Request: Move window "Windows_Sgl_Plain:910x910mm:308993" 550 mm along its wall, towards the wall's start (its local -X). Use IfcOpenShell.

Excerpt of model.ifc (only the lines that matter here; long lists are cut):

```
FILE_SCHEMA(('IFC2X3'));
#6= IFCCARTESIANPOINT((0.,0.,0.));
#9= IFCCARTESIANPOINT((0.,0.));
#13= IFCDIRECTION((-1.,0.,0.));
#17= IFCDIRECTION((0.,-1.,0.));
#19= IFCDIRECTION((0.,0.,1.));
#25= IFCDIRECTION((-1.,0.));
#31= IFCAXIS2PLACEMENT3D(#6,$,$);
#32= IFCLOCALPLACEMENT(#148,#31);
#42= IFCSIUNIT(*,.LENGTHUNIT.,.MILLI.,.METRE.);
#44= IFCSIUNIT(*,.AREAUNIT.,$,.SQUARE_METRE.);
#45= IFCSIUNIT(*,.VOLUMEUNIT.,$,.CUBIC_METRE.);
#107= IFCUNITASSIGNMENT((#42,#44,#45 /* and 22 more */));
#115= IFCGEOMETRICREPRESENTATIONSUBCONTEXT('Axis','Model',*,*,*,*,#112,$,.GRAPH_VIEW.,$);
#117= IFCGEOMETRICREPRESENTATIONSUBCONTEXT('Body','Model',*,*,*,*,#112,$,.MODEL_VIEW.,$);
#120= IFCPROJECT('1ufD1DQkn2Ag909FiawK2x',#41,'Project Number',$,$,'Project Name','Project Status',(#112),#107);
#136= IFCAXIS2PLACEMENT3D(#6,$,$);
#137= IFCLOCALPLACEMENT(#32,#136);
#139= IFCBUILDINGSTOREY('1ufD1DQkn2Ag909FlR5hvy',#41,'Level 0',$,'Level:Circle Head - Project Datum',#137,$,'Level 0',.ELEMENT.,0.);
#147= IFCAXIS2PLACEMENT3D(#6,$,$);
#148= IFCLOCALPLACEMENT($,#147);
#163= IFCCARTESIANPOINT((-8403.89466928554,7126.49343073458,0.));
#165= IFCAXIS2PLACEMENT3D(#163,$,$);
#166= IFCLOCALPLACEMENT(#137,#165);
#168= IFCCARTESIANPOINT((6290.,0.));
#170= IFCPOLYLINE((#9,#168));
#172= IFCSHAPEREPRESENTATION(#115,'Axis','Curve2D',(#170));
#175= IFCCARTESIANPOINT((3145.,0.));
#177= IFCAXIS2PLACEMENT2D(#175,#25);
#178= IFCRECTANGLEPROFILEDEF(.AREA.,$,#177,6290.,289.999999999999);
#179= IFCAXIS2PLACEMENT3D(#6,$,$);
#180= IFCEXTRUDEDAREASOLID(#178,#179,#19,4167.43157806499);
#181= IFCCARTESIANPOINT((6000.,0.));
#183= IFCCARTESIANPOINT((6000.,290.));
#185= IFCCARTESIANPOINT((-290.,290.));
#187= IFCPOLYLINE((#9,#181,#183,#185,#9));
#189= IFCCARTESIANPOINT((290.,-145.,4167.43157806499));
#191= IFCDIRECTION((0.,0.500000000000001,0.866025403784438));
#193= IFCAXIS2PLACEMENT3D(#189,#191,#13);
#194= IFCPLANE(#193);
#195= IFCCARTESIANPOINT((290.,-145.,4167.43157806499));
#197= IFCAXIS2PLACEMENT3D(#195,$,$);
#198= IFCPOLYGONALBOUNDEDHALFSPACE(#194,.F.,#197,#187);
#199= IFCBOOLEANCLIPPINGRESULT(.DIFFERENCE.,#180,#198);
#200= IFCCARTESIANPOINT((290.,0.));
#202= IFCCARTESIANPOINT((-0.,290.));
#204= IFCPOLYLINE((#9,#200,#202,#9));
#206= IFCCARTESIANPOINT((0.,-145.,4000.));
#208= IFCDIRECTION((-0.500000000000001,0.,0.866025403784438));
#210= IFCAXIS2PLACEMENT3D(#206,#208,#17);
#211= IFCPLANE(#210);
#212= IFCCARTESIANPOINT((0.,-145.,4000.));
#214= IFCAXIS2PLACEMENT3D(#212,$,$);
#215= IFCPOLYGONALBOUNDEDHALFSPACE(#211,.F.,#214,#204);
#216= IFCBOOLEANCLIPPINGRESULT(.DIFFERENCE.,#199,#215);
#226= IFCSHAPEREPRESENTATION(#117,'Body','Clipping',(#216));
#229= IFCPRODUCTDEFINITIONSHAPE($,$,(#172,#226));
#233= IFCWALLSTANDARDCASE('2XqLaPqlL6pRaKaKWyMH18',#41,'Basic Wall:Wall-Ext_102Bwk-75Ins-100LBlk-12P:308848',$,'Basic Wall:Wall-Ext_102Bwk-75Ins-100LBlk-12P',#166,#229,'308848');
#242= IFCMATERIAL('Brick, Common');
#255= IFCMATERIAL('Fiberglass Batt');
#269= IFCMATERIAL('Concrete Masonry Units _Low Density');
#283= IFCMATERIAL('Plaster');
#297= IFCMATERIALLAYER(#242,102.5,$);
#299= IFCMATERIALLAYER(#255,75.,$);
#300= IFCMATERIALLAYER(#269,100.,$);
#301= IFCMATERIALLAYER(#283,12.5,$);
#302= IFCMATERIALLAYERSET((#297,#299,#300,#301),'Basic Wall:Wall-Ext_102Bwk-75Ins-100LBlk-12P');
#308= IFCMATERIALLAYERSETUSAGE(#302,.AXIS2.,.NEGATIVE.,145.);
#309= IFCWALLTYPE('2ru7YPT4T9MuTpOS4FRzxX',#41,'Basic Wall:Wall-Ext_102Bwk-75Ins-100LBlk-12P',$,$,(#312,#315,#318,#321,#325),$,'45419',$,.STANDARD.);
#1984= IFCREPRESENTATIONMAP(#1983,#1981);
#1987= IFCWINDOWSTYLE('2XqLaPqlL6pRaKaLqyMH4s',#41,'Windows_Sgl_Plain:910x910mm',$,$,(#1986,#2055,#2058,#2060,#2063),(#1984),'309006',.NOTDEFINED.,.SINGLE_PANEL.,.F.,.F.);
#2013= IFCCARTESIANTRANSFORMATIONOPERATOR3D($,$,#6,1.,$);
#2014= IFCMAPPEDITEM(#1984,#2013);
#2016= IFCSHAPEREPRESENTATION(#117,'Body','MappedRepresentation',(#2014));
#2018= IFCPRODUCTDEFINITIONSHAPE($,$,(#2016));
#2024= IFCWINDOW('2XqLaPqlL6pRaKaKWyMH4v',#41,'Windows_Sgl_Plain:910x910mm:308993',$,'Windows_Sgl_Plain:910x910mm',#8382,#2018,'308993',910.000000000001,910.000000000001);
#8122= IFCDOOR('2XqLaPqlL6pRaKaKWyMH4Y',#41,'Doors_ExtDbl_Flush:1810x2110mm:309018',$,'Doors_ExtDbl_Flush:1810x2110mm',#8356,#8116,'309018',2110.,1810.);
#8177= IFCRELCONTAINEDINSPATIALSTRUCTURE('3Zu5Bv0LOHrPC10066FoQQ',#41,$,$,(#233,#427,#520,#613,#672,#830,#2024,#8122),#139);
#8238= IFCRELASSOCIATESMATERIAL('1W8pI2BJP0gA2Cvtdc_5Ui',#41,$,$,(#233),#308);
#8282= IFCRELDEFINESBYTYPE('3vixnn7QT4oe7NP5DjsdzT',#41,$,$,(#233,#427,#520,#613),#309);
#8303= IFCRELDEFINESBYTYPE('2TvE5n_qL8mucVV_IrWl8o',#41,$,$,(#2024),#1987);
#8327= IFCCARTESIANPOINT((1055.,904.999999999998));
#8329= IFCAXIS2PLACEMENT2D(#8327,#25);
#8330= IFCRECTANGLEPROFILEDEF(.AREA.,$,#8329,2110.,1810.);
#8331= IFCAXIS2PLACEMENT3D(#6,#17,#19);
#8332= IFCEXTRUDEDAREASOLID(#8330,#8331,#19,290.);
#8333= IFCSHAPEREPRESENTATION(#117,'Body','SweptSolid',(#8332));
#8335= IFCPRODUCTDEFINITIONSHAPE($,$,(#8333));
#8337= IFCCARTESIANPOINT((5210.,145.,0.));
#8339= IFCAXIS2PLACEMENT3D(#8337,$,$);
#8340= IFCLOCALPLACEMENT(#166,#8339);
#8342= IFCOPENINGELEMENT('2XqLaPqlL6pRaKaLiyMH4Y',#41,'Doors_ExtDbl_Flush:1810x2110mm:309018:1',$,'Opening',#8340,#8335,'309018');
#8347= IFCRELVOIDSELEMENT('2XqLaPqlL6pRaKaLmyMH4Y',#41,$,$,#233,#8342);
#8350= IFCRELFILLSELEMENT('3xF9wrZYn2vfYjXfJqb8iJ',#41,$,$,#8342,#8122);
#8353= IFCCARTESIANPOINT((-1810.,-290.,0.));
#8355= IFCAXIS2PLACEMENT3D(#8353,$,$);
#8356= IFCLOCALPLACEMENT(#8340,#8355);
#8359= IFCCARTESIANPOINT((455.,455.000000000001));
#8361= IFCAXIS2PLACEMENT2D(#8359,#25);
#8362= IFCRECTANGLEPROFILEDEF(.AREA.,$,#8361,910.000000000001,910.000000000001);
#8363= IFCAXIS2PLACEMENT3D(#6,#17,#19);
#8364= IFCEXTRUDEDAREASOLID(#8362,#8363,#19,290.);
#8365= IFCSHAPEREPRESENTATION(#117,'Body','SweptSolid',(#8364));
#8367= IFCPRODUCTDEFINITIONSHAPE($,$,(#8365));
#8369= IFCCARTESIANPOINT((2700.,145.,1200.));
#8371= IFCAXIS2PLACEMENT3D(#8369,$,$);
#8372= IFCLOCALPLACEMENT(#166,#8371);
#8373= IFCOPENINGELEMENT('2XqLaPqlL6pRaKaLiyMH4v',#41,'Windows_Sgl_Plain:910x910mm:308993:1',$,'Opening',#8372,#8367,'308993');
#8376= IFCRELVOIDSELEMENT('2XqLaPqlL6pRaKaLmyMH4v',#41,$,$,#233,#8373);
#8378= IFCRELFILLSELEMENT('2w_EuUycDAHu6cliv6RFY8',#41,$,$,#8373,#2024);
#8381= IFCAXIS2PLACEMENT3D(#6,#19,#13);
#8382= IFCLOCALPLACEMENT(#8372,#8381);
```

```python
import ifcopenshell
import ifcopenshell.api.geometry
import ifcopenshell.util.placement
import ifcopenshell.util.unit

model = ifcopenshell.open("model.ifc")
unit_scale = ifcopenshell.util.unit.calculate_unit_scale(model)

window = model.by_id(2024)
opening = window.FillsVoids[0].RelatingOpeningElement
wall = opening.VoidsElements[0].RelatingBuildingElement

wall_matrix = ifcopenshell.util.placement.get_local_placement(wall.ObjectPlacement)
shift = wall_matrix[:3, 0] * -0.55 / unit_scale
before = ifcopenshell.util.placement.get_local_placement(window.ObjectPlacement)[:3, 3].copy()

# The window is placed relative to its opening, so it follows when the opening moves.
matrix = ifcopenshell.util.placement.get_local_placement(opening.ObjectPlacement)
matrix[:3, 3] += shift
ifcopenshell.api.geometry.edit_object_placement(
    model, product=opening, matrix=matrix, is_si=False, should_transform_children=True
)

after = ifcopenshell.util.placement.get_local_placement(window.ObjectPlacement)[:3, 3]
print("window moved by", (after - before).round(3) + 0.0)

model.write("model_edited.ifc")
```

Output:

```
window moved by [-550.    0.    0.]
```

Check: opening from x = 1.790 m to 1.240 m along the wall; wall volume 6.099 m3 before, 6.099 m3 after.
